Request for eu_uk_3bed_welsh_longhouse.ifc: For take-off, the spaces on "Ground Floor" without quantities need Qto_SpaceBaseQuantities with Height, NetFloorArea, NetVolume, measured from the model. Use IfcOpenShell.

First a look at what the model holds.

```python
import ifcopenshell
import ifcopenshell.util.element
import ifcopenshell.util.unit

model = ifcopenshell.open("eu_uk_3bed_welsh_longhouse.ifc")
print(model.schema)
for unit_type in ("LENGTHUNIT", "AREAUNIT", "VOLUMEUNIT"):
    print(unit_type, ifcopenshell.util.unit.calculate_unit_scale(model, unit_type))
storey = next(s for s in model.by_type("IfcBuildingStorey") if s.Name == "Ground Floor")
spaces = [e for e in ifcopenshell.util.element.get_decomposition(storey) if e.is_a("IfcSpace")]
for e in sorted(spaces, key=lambda e: e.id()):
    print(e.id(), e.is_a(), e.Name, list(ifcopenshell.util.element.get_psets(e, qtos_only=True)), sep=" | ")
```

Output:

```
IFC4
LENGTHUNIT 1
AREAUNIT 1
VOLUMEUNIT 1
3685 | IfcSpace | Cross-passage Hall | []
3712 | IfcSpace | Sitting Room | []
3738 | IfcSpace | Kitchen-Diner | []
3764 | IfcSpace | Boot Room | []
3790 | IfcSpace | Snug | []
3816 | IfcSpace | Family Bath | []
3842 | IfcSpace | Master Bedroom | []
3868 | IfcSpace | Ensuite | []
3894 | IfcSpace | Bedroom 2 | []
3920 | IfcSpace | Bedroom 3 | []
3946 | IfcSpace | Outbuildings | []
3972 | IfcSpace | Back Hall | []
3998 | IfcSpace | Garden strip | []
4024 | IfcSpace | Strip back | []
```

```python
import ifcopenshell
import ifcopenshell.api.pset
import ifcopenshell.geom
import ifcopenshell.util.element
import ifcopenshell.util.shape
import ifcopenshell.util.unit

model = ifcopenshell.open("eu_uk_3bed_welsh_longhouse.ifc")
unit_scale = ifcopenshell.util.unit.calculate_unit_scale(model)
area_scale = ifcopenshell.util.unit.calculate_unit_scale(model, "AREAUNIT")
volume_scale = ifcopenshell.util.unit.calculate_unit_scale(model, "VOLUMEUNIT")
settings = ifcopenshell.geom.settings()

storey = next(s for s in model.by_type("IfcBuildingStorey") if s.Name == "Ground Floor")
spaces = [e for e in ifcopenshell.util.element.get_decomposition(storey) if e.is_a("IfcSpace")]

for e in sorted(spaces, key=lambda e: e.id()):
    if ifcopenshell.util.element.get_psets(e, qtos_only=True, should_inherit=False):
        continue
    # Geometry comes back in metres, in the element's own axes.
    shape = ifcopenshell.geom.create_shape(settings, e)
    values = {
        "Height": ifcopenshell.util.shape.get_z(shape.geometry) / unit_scale,
        "NetFloorArea": ifcopenshell.util.shape.get_footprint_area(shape.geometry) / area_scale,
        "NetVolume": ifcopenshell.util.shape.get_volume(shape.geometry) / volume_scale,
    }
    qto = ifcopenshell.api.pset.add_qto(model, product=e, name="Qto_SpaceBaseQuantities")
    ifcopenshell.api.pset.edit_qto(model, qto=qto, properties=values)
    print(e.id(), {k: round(v, 3) for k, v in values.items()})

model.write("eu_uk_3bed_welsh_longhouse_updated.ifc")
```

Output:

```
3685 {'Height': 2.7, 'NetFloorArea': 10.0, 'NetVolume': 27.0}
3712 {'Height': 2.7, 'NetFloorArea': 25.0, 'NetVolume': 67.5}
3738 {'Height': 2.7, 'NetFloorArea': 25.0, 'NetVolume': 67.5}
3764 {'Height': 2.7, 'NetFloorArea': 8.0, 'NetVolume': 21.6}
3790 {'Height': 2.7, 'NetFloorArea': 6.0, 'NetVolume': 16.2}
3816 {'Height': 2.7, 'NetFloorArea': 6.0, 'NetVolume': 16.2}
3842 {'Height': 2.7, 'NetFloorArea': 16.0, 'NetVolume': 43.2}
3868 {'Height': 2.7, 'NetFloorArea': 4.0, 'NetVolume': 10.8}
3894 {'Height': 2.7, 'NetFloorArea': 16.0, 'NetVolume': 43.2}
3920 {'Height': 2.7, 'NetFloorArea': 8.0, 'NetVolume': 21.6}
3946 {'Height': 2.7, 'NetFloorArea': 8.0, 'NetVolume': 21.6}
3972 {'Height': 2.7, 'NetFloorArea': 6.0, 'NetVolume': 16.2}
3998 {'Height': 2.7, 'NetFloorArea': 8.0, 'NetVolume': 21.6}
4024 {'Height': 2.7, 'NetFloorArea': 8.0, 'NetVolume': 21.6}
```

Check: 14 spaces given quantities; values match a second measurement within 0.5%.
